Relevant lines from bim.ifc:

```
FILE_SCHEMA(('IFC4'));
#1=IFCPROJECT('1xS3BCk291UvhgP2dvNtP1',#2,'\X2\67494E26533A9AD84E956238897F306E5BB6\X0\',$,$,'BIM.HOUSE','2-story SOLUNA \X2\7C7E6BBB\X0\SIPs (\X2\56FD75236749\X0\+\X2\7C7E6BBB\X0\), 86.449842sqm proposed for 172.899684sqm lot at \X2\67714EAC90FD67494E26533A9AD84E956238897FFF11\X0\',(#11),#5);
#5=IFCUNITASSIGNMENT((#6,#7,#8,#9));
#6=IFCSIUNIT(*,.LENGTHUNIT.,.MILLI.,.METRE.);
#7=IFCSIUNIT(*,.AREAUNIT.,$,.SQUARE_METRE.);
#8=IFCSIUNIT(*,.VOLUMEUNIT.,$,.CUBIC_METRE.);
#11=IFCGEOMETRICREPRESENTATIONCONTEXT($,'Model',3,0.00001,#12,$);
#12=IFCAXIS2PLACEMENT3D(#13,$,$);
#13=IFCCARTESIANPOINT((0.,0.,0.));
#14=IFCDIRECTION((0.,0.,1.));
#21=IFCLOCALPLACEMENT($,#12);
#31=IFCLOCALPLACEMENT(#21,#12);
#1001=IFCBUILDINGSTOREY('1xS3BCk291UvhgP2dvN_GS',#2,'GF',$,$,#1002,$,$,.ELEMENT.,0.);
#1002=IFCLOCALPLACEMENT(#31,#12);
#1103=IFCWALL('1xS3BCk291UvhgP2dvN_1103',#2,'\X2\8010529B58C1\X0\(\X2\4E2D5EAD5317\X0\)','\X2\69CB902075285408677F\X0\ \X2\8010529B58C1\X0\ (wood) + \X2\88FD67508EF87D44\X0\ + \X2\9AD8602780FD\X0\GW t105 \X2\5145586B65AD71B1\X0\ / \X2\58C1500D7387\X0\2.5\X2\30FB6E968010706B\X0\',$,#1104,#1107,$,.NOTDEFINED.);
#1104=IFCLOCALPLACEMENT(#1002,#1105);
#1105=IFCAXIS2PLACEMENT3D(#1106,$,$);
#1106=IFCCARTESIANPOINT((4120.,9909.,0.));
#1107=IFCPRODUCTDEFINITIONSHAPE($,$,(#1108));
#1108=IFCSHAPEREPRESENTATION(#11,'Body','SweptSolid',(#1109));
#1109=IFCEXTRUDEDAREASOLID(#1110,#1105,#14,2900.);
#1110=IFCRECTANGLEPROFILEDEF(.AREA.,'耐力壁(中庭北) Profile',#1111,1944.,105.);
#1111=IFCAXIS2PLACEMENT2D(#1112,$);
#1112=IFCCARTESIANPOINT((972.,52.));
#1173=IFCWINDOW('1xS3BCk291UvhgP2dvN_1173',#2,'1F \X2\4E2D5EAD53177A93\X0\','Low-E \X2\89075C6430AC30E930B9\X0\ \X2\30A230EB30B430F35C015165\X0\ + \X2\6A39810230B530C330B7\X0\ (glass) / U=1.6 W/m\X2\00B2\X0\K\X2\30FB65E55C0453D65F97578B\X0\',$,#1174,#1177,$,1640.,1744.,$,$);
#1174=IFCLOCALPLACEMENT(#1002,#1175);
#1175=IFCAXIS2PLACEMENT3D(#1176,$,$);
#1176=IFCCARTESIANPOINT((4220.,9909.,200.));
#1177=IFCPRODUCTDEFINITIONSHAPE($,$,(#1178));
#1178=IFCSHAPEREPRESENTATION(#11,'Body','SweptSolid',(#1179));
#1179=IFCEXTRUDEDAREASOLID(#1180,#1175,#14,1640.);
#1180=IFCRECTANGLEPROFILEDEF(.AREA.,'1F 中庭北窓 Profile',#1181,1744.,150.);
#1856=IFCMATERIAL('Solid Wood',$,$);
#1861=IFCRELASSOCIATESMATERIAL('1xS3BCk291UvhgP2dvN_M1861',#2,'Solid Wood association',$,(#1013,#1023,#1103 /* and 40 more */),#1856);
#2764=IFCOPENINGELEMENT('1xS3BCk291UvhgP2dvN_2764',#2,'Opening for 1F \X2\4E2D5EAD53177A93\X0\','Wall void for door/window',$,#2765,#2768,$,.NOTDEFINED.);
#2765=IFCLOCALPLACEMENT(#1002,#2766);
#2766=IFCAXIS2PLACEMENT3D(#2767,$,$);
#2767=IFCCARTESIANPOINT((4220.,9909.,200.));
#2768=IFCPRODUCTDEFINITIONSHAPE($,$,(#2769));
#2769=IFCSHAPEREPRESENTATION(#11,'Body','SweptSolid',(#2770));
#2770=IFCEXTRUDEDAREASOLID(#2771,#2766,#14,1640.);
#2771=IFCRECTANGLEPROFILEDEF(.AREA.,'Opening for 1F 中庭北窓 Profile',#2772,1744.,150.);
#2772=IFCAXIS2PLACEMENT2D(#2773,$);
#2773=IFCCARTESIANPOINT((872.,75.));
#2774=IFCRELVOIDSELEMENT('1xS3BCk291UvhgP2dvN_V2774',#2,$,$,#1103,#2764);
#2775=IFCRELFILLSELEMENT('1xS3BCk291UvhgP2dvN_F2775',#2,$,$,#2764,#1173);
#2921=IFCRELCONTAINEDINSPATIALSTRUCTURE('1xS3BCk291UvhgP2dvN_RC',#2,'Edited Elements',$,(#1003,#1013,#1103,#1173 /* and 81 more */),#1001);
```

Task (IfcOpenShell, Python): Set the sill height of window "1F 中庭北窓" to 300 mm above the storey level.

```python
import numpy as np
import ifcopenshell
import ifcopenshell.api.geometry
import ifcopenshell.geom
import ifcopenshell.util.element
import ifcopenshell.util.placement
import ifcopenshell.util.shape
import ifcopenshell.util.unit

model = ifcopenshell.open("bim.ifc")
unit_scale = ifcopenshell.util.unit.calculate_unit_scale(model)

window = model.by_id(1173)
opening = window.FillsVoids[0].RelatingOpeningElement
storey = ifcopenshell.util.element.get_container(window, ifc_class="IfcBuildingStorey")
level = ifcopenshell.util.placement.get_local_placement(storey.ObjectPlacement)[2, 3]

# The opening's origin need not be at the sill, so measure its lowest point.
shape = ifcopenshell.geom.create_shape(ifcopenshell.geom.settings(), opening)
bottom = ifcopenshell.util.shape.get_shape_bottom_elevation(shape, shape.geometry) / unit_scale
dz = level + 300.0 - bottom

shift = np.array([0.0, 0.0, dz])
# The window is not placed relative to its opening, so move both.
for product in (opening, window):
    matrix = ifcopenshell.util.placement.get_local_placement(product.ObjectPlacement)
    matrix[:3, 3] += shift
    ifcopenshell.api.geometry.edit_object_placement(model, product=product, matrix=matrix, is_si=False)

print(f"moved by {dz * unit_scale:+.3f} m")

model.write("bim_v2.ifc")
```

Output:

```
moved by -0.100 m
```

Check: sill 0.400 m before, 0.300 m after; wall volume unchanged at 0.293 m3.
